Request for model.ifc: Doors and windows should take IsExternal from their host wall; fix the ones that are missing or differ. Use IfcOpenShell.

First a look at what the model holds.

```python
import ifcopenshell
import ifcopenshell.util.element

model = ifcopenshell.open("model.ifc")
print(model.schema)
seen = {}
for e in model.by_type("IfcDoor") + model.by_type("IfcWindow"):
    if not e.FillsVoids:
        continue
    host = e.FillsVoids[0].RelatingOpeningElement.VoidsElements[0].RelatingBuildingElement
    own = ifcopenshell.util.element.get_pset(e, f"Pset_{e.is_a()[3:].removesuffix('StandardCase')}Common", "IsExternal")
    wall = ifcopenshell.util.element.get_pset(host, "Pset_WallCommon", "IsExternal")
    seen[e.is_a(), own, wall] = seen.get((e.is_a(), own, wall), 0) + 1
for (cls, own, wall), count in sorted(seen.items(), key=str):
    print(count, cls, "IsExternal:", own, "| host wall:", wall)
```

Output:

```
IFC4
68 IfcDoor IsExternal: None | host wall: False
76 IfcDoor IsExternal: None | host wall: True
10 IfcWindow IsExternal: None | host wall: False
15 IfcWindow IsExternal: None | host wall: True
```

```python
import ifcopenshell
import ifcopenshell.api.pset
import ifcopenshell.util.element

model = ifcopenshell.open("model.ifc")

count = 0
for ifc_class, pset_name in (("IfcDoor", "Pset_DoorCommon"), ("IfcWindow", "Pset_WindowCommon")):
    for e in model.by_type(ifc_class):
        if not e.FillsVoids:
            continue
        host = e.FillsVoids[0].RelatingOpeningElement.VoidsElements[0].RelatingBuildingElement
        external = ifcopenshell.util.element.get_pset(host, "Pset_WallCommon", "IsExternal")
        if external is None or ifcopenshell.util.element.get_pset(e, pset_name, "IsExternal") == external:
            continue
        pset = ifcopenshell.api.pset.add_pset(model, product=e, name=pset_name)
        ifcopenshell.api.pset.edit_pset(model, pset=pset, properties={"IsExternal": external})
        count += 1

print(count, "updated")

model.write("model_rev.ifc")
```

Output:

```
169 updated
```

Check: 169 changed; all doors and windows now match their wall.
